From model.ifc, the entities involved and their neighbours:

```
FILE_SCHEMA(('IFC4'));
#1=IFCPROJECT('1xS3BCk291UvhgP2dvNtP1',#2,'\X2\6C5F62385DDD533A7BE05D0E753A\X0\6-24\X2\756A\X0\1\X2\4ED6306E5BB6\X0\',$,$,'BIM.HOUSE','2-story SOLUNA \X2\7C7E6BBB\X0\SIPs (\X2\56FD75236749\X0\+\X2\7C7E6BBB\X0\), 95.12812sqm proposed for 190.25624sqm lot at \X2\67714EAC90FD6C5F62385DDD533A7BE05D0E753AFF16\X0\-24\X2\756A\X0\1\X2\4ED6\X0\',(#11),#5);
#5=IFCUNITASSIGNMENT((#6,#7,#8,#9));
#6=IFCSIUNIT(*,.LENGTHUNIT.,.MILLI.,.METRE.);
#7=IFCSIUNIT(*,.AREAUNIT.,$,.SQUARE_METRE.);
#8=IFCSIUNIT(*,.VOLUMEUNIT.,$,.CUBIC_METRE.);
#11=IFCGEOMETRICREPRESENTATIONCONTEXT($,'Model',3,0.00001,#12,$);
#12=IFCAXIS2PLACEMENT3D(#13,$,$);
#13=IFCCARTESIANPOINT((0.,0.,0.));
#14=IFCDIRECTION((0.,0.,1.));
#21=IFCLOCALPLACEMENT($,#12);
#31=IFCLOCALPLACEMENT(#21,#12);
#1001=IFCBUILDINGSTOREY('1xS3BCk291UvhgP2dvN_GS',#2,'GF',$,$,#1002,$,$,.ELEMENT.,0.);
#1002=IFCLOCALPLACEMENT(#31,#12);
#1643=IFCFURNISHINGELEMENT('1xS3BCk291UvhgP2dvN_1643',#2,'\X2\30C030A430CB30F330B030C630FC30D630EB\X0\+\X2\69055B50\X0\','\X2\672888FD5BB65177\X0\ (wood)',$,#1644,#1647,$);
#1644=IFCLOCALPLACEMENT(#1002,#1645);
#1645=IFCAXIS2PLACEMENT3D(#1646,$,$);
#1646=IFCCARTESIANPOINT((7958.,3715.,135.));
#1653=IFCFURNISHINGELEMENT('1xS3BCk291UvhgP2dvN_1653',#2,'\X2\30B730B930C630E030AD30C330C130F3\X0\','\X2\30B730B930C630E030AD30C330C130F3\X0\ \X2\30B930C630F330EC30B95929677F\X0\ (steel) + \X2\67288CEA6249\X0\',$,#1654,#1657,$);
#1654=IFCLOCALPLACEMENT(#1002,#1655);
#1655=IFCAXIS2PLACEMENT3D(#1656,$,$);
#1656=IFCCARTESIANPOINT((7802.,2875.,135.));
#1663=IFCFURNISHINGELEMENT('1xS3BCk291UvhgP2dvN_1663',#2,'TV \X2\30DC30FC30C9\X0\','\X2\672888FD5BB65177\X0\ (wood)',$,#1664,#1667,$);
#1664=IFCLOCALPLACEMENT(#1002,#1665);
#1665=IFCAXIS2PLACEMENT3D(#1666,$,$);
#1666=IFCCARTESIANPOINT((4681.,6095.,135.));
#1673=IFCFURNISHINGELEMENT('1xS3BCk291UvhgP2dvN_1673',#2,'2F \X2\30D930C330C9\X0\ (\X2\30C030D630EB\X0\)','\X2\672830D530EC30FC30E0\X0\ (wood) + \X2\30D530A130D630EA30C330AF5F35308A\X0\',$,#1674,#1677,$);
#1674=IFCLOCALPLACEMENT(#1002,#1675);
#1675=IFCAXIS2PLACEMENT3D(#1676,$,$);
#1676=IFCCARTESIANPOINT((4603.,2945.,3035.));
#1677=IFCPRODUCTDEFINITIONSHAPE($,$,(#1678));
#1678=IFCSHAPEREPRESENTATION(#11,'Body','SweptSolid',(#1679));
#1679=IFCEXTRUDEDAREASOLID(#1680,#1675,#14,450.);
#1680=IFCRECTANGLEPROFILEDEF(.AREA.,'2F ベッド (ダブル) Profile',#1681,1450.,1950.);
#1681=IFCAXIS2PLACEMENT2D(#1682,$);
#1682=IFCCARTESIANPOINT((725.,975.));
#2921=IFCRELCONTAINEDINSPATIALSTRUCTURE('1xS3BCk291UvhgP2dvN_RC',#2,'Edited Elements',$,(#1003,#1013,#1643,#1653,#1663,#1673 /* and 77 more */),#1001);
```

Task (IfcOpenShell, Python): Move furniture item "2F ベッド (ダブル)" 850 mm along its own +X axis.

```python
import ifcopenshell
import ifcopenshell.api.geometry
import ifcopenshell.util.placement

model = ifcopenshell.open("model.ifc")

item = model.by_guid("1xS3BCk291UvhgP2dvN_1673")
matrix = ifcopenshell.util.placement.get_local_placement(item.ObjectPlacement)
matrix[:3, 3] += matrix[:3, 0] * 850.0
ifcopenshell.api.geometry.edit_object_placement(model, product=item, matrix=matrix, is_si=False)

print(ifcopenshell.util.placement.get_local_placement(item.ObjectPlacement).round(3) + 0.0)

model.write("model_updated.ifc")
```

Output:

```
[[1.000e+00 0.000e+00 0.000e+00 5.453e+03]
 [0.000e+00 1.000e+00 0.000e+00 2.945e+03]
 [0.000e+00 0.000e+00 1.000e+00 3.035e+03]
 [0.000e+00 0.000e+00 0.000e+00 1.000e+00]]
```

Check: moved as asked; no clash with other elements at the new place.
